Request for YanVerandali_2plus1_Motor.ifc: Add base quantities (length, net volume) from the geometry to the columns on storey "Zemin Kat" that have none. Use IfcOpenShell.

First a look at what the model holds.

```python
import ifcopenshell
import ifcopenshell.util.element
import ifcopenshell.util.unit

model = ifcopenshell.open("YanVerandali_2plus1_Motor.ifc")
print(model.schema)
for unit_type in ("LENGTHUNIT", "AREAUNIT", "VOLUMEUNIT"):
    print(unit_type, ifcopenshell.util.unit.calculate_unit_scale(model, unit_type))
storey = next(s for s in model.by_type("IfcBuildingStorey") if s.Name == "Zemin Kat")
columns = [e for e in ifcopenshell.util.element.get_decomposition(storey) if e.is_a("IfcColumn")]
for e in sorted(columns, key=lambda e: e.id()):
    print(e.id(), e.is_a(), e.Name, list(ifcopenshell.util.element.get_psets(e, qtos_only=True)), sep=" | ")
```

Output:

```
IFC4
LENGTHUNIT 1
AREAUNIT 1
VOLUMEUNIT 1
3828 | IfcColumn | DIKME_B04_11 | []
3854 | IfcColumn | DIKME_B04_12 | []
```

```python
import ifcopenshell
import ifcopenshell.api.pset
import ifcopenshell.geom
import ifcopenshell.util.element
import ifcopenshell.util.shape
import ifcopenshell.util.unit

model = ifcopenshell.open("YanVerandali_2plus1_Motor.ifc")
unit_scale = ifcopenshell.util.unit.calculate_unit_scale(model)
volume_scale = ifcopenshell.util.unit.calculate_unit_scale(model, "VOLUMEUNIT")
settings = ifcopenshell.geom.settings()

storey = next(s for s in model.by_type("IfcBuildingStorey") if s.Name == "Zemin Kat")
columns = [e for e in ifcopenshell.util.element.get_decomposition(storey) if e.is_a("IfcColumn")]

for e in sorted(columns, key=lambda e: e.id()):
    if ifcopenshell.util.element.get_psets(e, qtos_only=True, should_inherit=False):
        continue
    # Geometry comes back in metres, in the element's own axes.
    shape = ifcopenshell.geom.create_shape(settings, e)
    values = {
        "Length": ifcopenshell.util.shape.get_z(shape.geometry) / unit_scale,
        "NetVolume": ifcopenshell.util.shape.get_volume(shape.geometry) / volume_scale,
    }
    qto = ifcopenshell.api.pset.add_qto(model, product=e, name="Qto_ColumnBaseQuantities")
    ifcopenshell.api.pset.edit_qto(model, qto=qto, properties=values)
    print(e.id(), {k: round(v, 3) for k, v in values.items()})

model.write("YanVerandali_2plus1_Motor-out.ifc")
```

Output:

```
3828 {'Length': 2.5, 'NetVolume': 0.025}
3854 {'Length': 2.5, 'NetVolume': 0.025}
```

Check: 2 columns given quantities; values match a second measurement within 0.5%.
